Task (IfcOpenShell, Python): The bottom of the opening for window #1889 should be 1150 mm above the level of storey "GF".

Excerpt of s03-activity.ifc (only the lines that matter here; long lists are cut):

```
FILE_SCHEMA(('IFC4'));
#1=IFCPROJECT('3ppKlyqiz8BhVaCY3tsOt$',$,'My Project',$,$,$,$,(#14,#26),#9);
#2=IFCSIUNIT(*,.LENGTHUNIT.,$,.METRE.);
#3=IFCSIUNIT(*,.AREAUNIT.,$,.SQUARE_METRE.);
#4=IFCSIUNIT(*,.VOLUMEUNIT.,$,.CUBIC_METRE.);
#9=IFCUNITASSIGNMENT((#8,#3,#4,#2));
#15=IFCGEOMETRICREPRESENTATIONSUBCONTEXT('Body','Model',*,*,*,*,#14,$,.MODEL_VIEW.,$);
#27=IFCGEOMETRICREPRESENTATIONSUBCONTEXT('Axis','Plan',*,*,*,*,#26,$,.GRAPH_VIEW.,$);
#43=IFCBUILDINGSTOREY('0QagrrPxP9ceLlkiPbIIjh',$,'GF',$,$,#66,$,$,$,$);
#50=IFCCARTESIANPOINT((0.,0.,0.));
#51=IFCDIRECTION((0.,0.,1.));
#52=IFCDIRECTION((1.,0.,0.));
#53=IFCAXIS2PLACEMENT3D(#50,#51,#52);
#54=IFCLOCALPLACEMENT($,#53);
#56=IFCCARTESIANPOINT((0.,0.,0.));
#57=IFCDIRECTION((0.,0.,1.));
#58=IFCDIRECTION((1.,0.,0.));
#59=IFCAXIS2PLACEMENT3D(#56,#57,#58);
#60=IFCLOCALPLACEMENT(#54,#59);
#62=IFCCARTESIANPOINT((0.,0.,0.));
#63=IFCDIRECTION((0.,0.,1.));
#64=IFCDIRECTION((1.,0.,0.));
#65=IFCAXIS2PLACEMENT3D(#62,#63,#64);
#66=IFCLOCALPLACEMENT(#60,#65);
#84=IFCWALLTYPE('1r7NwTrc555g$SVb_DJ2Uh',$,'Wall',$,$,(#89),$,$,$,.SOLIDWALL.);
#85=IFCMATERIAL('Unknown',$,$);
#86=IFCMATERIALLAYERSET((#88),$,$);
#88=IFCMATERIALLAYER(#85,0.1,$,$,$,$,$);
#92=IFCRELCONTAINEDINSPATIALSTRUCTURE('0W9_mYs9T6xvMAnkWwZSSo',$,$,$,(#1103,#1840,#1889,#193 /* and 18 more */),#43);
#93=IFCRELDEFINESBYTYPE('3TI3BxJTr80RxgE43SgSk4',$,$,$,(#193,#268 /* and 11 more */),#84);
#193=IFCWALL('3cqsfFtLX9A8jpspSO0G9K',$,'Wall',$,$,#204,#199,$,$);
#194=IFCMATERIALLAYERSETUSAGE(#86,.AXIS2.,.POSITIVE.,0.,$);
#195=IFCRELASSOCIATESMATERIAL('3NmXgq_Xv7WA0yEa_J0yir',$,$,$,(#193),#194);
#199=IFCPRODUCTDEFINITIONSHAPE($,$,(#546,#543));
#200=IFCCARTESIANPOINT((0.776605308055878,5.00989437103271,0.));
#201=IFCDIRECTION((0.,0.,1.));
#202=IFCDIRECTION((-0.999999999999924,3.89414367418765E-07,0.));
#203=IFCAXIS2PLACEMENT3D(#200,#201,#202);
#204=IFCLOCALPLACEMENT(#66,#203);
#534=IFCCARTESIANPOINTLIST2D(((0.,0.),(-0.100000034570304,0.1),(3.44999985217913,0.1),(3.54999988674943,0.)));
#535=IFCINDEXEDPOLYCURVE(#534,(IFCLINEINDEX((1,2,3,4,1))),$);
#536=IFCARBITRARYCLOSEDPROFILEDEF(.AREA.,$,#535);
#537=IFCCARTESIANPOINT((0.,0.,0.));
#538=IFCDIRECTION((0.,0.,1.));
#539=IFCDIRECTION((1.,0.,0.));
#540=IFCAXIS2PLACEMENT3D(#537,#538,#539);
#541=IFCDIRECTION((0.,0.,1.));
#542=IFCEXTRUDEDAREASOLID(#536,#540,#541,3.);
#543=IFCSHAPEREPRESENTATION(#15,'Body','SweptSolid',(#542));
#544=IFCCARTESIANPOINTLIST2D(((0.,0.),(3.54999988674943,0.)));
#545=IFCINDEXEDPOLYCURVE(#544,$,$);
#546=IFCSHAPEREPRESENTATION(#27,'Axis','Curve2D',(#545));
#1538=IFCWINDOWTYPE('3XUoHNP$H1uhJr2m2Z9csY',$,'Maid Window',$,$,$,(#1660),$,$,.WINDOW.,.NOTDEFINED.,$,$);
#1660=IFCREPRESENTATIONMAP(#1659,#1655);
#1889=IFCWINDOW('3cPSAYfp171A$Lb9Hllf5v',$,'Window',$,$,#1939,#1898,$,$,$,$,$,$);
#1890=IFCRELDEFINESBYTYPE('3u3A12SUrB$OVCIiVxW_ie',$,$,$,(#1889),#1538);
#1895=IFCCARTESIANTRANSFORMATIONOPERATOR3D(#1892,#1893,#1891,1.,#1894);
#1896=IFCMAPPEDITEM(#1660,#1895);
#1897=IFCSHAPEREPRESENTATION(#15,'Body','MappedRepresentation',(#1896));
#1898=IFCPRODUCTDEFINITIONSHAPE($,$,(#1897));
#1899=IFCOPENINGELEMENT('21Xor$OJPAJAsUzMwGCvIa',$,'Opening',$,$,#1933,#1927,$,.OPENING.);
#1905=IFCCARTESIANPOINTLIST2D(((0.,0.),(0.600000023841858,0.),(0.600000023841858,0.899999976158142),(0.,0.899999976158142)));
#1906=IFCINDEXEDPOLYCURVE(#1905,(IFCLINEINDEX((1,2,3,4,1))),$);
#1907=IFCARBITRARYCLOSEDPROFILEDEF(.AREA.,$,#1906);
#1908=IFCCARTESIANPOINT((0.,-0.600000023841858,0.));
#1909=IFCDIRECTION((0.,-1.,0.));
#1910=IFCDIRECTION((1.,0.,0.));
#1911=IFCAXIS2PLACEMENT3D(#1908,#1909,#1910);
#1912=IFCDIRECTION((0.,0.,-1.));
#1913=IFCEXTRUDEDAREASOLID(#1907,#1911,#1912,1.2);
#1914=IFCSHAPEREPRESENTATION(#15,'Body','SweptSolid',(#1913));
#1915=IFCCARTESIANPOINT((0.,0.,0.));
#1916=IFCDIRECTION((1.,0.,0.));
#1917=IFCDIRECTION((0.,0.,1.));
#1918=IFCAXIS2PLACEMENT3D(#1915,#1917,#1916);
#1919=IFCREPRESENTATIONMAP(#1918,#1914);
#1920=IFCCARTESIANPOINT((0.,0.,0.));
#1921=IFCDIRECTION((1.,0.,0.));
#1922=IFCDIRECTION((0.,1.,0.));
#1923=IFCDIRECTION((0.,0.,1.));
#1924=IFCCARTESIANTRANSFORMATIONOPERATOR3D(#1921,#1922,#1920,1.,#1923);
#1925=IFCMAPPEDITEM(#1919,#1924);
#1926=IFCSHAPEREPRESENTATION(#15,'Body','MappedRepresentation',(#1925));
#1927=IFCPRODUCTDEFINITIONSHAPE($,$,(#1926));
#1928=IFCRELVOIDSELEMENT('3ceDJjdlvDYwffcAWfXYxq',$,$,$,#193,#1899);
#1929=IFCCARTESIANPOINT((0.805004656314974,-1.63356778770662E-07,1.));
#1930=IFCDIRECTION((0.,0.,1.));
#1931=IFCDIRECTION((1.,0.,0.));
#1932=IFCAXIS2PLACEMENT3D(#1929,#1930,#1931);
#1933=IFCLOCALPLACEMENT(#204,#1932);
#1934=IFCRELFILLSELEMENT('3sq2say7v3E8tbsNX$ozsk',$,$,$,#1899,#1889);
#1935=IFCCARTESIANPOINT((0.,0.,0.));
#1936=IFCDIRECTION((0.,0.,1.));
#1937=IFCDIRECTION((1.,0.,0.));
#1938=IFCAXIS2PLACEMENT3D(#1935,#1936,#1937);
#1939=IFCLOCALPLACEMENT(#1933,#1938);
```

```python
import numpy as np
import ifcopenshell
import ifcopenshell.api.geometry
import ifcopenshell.geom
import ifcopenshell.util.element
import ifcopenshell.util.placement
import ifcopenshell.util.shape
import ifcopenshell.util.unit

model = ifcopenshell.open("s03-activity.ifc")
unit_scale = ifcopenshell.util.unit.calculate_unit_scale(model)

window = model.by_guid("3cPSAYfp171A$Lb9Hllf5v")
opening = window.FillsVoids[0].RelatingOpeningElement
storey = ifcopenshell.util.element.get_container(window, ifc_class="IfcBuildingStorey")
level = ifcopenshell.util.placement.get_local_placement(storey.ObjectPlacement)[2, 3]

# The opening's origin need not be at the sill, so measure its lowest point.
shape = ifcopenshell.geom.create_shape(ifcopenshell.geom.settings(), opening)
bottom = ifcopenshell.util.shape.get_shape_bottom_elevation(shape, shape.geometry) / unit_scale
dz = level + 1.15 / unit_scale - bottom

shift = np.array([0.0, 0.0, dz])
# The window is placed relative to its opening, so it follows when the opening moves.
matrix = ifcopenshell.util.placement.get_local_placement(opening.ObjectPlacement)
matrix[:3, 3] += shift
ifcopenshell.api.geometry.edit_object_placement(
    model, product=opening, matrix=matrix, is_si=False, should_transform_children=True
)

print(f"moved by {dz * unit_scale:+.3f} m")

model.write("s03-activity_updated.ifc")
```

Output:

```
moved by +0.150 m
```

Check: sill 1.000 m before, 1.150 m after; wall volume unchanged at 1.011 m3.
